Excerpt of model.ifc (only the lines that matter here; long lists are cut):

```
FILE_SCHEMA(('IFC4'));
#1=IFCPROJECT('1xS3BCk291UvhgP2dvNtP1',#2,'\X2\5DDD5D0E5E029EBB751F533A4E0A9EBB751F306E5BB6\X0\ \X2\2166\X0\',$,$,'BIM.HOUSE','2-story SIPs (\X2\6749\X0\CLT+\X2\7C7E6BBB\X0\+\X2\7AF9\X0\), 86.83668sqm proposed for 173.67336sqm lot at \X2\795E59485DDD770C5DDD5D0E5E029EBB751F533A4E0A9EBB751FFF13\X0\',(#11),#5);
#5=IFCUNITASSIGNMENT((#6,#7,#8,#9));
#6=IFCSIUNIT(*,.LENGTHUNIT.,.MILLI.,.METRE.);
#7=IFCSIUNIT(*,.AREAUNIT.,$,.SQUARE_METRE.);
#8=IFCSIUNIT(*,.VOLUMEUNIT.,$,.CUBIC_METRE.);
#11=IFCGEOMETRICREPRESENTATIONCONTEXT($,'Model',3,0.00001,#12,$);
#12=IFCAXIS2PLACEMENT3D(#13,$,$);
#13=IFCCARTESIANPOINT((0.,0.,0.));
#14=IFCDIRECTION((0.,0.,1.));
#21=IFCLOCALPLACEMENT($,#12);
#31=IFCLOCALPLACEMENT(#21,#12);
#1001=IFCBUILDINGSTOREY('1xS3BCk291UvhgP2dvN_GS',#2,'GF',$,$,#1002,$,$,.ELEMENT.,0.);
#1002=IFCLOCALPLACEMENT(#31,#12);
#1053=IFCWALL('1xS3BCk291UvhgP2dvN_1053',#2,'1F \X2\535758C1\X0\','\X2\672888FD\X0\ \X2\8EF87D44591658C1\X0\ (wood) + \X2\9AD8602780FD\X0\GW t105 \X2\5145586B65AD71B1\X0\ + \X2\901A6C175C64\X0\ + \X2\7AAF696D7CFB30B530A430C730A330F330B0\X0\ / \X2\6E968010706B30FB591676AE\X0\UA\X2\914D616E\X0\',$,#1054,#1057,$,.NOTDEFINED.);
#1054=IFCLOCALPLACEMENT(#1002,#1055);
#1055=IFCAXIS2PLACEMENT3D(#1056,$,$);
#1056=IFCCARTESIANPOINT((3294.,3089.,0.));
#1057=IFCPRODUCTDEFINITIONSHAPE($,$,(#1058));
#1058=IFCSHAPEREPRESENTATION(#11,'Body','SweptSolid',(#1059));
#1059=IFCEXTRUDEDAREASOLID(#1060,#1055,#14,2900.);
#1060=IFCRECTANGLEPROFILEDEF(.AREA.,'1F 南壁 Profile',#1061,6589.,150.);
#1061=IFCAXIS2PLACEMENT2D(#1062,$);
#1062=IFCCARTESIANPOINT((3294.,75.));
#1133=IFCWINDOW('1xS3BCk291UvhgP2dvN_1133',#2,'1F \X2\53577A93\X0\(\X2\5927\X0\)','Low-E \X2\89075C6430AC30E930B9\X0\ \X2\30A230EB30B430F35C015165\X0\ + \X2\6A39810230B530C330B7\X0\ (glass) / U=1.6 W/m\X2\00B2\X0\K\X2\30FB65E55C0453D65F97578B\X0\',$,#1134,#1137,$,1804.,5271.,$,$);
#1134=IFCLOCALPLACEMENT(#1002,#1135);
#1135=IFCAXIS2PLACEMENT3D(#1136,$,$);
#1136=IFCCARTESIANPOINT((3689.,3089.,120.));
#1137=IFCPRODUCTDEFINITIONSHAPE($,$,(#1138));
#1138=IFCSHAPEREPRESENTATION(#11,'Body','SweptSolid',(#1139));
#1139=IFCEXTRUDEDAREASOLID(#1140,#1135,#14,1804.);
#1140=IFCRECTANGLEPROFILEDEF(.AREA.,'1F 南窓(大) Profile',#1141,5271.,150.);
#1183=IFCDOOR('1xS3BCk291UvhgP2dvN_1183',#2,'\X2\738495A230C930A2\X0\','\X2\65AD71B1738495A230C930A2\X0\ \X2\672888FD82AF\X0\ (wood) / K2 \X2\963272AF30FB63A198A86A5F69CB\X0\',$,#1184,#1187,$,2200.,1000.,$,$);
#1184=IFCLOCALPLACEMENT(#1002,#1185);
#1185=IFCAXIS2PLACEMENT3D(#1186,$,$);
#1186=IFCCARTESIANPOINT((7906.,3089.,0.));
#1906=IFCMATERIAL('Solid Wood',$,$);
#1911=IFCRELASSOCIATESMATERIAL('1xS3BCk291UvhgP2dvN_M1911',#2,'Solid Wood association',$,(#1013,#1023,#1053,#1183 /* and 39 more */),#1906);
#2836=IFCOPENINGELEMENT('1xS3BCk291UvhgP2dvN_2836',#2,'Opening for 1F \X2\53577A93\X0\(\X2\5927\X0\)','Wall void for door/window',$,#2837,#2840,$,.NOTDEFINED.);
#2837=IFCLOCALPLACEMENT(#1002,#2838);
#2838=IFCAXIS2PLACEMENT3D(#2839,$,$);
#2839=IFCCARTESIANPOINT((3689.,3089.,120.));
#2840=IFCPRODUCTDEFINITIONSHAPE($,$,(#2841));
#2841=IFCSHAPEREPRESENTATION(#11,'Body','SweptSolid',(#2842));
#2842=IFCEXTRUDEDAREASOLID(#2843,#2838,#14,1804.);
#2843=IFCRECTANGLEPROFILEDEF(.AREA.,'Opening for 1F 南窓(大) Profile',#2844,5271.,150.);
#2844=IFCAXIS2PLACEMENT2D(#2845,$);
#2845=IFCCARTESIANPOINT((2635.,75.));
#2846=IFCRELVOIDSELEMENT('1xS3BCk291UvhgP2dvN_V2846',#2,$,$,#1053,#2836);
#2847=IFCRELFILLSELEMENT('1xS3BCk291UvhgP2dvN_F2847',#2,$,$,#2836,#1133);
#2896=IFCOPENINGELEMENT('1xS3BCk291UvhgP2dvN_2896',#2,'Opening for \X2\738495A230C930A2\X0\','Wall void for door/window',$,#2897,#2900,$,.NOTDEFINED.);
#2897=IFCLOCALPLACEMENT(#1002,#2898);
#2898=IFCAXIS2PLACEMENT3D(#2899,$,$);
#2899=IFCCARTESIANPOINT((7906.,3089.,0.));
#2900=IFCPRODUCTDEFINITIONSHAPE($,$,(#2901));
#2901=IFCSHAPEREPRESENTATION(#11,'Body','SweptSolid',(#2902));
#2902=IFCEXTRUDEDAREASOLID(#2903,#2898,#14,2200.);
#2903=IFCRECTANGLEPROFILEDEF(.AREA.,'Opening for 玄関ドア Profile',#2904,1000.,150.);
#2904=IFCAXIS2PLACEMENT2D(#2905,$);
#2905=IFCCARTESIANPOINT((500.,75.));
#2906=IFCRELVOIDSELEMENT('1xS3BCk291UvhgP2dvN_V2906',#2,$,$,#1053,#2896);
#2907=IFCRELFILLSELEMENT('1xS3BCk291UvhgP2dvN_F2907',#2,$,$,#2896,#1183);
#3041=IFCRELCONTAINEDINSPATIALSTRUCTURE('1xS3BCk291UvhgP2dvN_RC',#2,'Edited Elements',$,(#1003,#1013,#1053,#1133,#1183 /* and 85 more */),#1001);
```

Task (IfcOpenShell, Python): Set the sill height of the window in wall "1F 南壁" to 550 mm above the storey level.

```python
import numpy as np
import ifcopenshell
import ifcopenshell.api.geometry
import ifcopenshell.geom
import ifcopenshell.util.element
import ifcopenshell.util.placement
import ifcopenshell.util.shape
import ifcopenshell.util.unit

model = ifcopenshell.open("model.ifc")
unit_scale = ifcopenshell.util.unit.calculate_unit_scale(model)

window = model.by_id(1133)
opening = window.FillsVoids[0].RelatingOpeningElement
storey = ifcopenshell.util.element.get_container(window, ifc_class="IfcBuildingStorey")
level = ifcopenshell.util.placement.get_local_placement(storey.ObjectPlacement)[2, 3]

# The opening's origin need not be at the sill, so measure its lowest point.
shape = ifcopenshell.geom.create_shape(ifcopenshell.geom.settings(), opening)
bottom = ifcopenshell.util.shape.get_shape_bottom_elevation(shape, shape.geometry) / unit_scale
dz = level + 550.0 - bottom

shift = np.array([0.0, 0.0, dz])
# The window is not placed relative to its opening, so move both.
for product in (opening, window):
    matrix = ifcopenshell.util.placement.get_local_placement(product.ObjectPlacement)
    matrix[:3, 3] += shift
    ifcopenshell.api.geometry.edit_object_placement(model, product=product, matrix=matrix, is_si=False)

print(f"moved by {dz * unit_scale:+.3f} m")

model.write("model_v2.ifc")
```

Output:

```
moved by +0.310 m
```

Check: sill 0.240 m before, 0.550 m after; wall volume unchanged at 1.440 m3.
